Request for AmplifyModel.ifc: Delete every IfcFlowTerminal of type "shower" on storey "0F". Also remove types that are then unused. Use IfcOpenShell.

First a look at what the model holds.

```python
import ifcopenshell
import ifcopenshell.util.element

model = ifcopenshell.open("AmplifyModel.ifc")
print(model.schema)
storey = next(s for s in model.by_type("IfcBuildingStorey") if s.Name == "0F")
terminals = [e for e in ifcopenshell.util.element.get_decomposition(storey) if e.is_a("IfcFlowTerminal")]
seen = {}
for e in terminals:
    element_type = ifcopenshell.util.element.get_type(e)
    name = element_type.Name if element_type not in (None, e) else None
    seen[name] = seen.get(name, 0) + 1
for name, count in sorted(seen.items(), key=str):
    print(count, "x", name)
```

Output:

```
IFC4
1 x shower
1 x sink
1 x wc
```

```python
import ifcopenshell
import ifcopenshell.api.root
import ifcopenshell.util.element

model = ifcopenshell.open("AmplifyModel.ifc")

storey = next(s for s in model.by_type("IfcBuildingStorey") if s.Name == "0F")
terminals = [e for e in ifcopenshell.util.element.get_decomposition(storey) if e.is_a("IfcFlowTerminal")]
targets = [e for e in terminals if (t := ifcopenshell.util.element.get_type(e)) not in (None, e) and t.Name == "shower"]
types = {ifcopenshell.util.element.get_type(e) for e in targets} - {None, *targets}

for e in targets:
    ifcopenshell.api.root.remove_product(model, product=e)
print(len(targets), "removed")

unused = [t for t in types if not ifcopenshell.util.element.get_types(t)]
for t in unused:
    ifcopenshell.api.root.remove_product(model, product=t)
print(len(unused), "unused types removed")

model.write("AmplifyModel_updated.ifc")
```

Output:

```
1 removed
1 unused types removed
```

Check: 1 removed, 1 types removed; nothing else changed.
